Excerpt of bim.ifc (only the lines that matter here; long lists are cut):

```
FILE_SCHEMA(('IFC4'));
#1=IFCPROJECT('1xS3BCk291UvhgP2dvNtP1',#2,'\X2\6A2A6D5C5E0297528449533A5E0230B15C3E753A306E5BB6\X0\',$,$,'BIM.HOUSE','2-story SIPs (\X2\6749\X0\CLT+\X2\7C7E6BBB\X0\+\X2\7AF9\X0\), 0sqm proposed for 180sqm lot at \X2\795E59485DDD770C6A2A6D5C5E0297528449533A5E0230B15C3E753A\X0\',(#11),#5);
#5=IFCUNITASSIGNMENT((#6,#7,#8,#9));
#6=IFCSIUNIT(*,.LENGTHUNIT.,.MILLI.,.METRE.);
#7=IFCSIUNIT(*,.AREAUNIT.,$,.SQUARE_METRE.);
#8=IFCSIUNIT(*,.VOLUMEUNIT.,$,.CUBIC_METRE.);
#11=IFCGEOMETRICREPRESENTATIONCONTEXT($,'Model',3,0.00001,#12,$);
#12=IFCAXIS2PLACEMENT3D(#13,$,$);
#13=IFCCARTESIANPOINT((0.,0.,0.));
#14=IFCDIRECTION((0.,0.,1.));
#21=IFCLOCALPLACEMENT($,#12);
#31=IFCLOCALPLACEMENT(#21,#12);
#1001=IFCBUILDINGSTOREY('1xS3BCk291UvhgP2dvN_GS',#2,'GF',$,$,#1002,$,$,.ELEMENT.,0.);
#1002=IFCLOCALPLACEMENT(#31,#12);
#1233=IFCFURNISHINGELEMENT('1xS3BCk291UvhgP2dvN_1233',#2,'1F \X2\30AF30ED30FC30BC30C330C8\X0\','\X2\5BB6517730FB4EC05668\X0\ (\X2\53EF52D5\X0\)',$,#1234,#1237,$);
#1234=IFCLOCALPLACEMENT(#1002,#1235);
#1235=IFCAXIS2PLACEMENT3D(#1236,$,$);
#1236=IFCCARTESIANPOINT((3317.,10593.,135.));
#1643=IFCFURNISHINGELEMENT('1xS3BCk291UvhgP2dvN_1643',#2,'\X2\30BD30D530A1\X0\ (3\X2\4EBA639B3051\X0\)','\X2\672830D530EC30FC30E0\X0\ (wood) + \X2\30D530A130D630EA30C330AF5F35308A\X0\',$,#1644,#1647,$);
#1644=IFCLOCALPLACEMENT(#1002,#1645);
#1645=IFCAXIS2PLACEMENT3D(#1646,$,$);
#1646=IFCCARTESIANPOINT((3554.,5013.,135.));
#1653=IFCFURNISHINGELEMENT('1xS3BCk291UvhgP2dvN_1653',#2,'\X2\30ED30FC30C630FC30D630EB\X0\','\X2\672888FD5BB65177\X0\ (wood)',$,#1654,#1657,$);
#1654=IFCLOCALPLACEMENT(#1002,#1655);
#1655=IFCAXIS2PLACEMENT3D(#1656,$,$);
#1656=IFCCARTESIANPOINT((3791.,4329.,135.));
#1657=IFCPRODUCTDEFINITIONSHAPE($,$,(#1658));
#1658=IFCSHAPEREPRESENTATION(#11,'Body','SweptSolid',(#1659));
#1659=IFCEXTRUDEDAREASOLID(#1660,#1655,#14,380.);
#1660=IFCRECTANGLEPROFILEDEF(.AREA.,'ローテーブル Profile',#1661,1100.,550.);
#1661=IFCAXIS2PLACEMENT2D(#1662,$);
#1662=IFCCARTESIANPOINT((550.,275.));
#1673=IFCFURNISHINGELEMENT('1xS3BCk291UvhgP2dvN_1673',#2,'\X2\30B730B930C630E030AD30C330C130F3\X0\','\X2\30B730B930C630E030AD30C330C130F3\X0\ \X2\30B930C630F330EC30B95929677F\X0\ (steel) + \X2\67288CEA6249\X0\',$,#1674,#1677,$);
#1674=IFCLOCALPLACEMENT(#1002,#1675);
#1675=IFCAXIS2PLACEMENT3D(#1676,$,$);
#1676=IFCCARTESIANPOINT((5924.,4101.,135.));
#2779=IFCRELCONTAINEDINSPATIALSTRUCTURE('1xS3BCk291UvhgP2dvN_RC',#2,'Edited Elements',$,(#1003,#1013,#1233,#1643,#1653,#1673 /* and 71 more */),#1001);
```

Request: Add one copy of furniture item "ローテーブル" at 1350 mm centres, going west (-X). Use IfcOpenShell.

```python
import numpy as np
import ifcopenshell
import ifcopenshell.api.geometry
import ifcopenshell.api.root
import ifcopenshell.util.element
import ifcopenshell.util.placement
import ifcopenshell.util.unit

model = ifcopenshell.open("bim.ifc")
unit_scale = ifcopenshell.util.unit.calculate_unit_scale(model)


def reuse_history(source, copy):
    """copy_class also copies each property set's owner history, people and application; keep the originals."""
    for rel in copy.IsDefinedBy:
        if rel.is_a("IfcRelDefinesByProperties") and (history := rel.RelatingPropertyDefinition.OwnerHistory):
            rel.RelatingPropertyDefinition.OwnerHistory = source.OwnerHistory
            ifcopenshell.util.element.remove_deep2(model, history)


source = model.by_id(1653)
base = ifcopenshell.util.placement.get_local_placement(source.ObjectPlacement)
step = np.array([-1.0, 0.0, 0.0]) * 1.35 / unit_scale

for i in range(1, 2):
    copy = ifcopenshell.api.root.copy_class(model, product=source)
    copy.Representation = ifcopenshell.util.element.copy_deep(
        model, source.Representation, exclude=["IfcGeometricRepresentationContext", "IfcRepresentationMap"]
    )
    reuse_history(source, copy)
    matrix = base.copy()
    matrix[:3, 3] += i * step
    print("added at", matrix[:3, 3].round(3) + 0.0)
    ifcopenshell.api.geometry.edit_object_placement(model, product=copy, matrix=matrix, is_si=False)

model.write("bim-out.ifc")
```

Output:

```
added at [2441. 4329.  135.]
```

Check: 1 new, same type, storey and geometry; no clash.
